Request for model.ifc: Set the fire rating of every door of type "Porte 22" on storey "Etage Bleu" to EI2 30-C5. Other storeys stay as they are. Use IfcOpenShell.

First a look at what the model holds.

```python
import ifcopenshell
import ifcopenshell.util.element

model = ifcopenshell.open("model.ifc")
print(model.schema)
storey = next(s for s in model.by_type("IfcBuildingStorey") if s.Name == "Etage Bleu")
doors = [e for e in ifcopenshell.util.element.get_decomposition(storey) if e.is_a("IfcDoor")]
seen = {}
for e in doors:
    element_type = ifcopenshell.util.element.get_type(e)
    key = (element_type.Name if element_type != e and element_type else None, ifcopenshell.util.element.get_pset(e, "Pset_DoorCommon", "FireRating"))
    seen[key] = seen.get(key, 0) + 1
for (name, value), count in sorted(seen.items(), key=str):
    print(count, "x", name, "|", value)
```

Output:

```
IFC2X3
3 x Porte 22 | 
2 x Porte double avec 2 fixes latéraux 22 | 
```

```python
import ifcopenshell
import ifcopenshell.api.pset
import ifcopenshell.util.element

model = ifcopenshell.open("model.ifc")

storey = next(s for s in model.by_type("IfcBuildingStorey") if s.Name == "Etage Bleu")
doors = [e for e in ifcopenshell.util.element.get_decomposition(storey) if e.is_a("IfcDoor")]

count = 0
for e in doors:
    element_type = ifcopenshell.util.element.get_type(e)
    if element_type in (None, e) or element_type.Name != "Porte 22":
        continue
    # add_pset returns the element's existing set when there is one.
    pset = ifcopenshell.api.pset.add_pset(model, product=e, name="Pset_DoorCommon")
    ifcopenshell.api.pset.edit_pset(model, pset=pset, properties={"FireRating": "EI2 30-C5"})
    count += 1

print(count, "doors updated")

model.write("model_updated.ifc")
```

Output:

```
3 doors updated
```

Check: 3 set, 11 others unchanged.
